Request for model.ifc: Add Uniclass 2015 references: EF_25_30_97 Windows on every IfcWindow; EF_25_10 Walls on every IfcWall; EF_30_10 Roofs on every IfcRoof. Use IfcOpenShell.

First a look at what the model holds.

```python
import ifcopenshell

model = ifcopenshell.open("model.ifc")
print(model.schema)
print("classifications:", [c.Name for c in model.by_type("IfcClassification")])
for ifc_class in ("IfcDoor", "IfcRoof", "IfcStair", "IfcWall", "IfcWindow"):
    print(ifc_class, len(model.by_type(ifc_class)))
```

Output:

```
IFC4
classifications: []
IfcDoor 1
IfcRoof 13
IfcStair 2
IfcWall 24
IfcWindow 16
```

```python
import ifcopenshell
import ifcopenshell.api.classification

model = ifcopenshell.open("model.ifc")

system = ifcopenshell.api.classification.add_classification(model, classification="Uniclass 2015")

codes = {
    "IfcWindow": ("EF_25_30_97", "Windows"),
    "IfcWall": ("EF_25_10", "Walls"),
    "IfcRoof": ("EF_30_10", "Roofs"),
}
for ifc_class, (code, name) in codes.items():
    products = model.by_type(ifc_class)
    ifcopenshell.api.classification.add_reference(
        model, products=products, classification=system, identification=code, name=name
    )
    print(code, len(products))

model.write("model_rev.ifc")
```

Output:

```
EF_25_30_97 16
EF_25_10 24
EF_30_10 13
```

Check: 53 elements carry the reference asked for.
